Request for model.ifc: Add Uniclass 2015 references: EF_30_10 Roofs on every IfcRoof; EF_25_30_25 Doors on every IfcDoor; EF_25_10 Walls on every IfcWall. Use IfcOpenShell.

First a look at what the model holds.

```python
import ifcopenshell

model = ifcopenshell.open("model.ifc")
print(model.schema)
print("classifications:", [c.Name for c in model.by_type("IfcClassification")])
for ifc_class in ("IfcDoor", "IfcRoof", "IfcStair", "IfcWall", "IfcWindow"):
    print(ifc_class, len(model.by_type(ifc_class)))
```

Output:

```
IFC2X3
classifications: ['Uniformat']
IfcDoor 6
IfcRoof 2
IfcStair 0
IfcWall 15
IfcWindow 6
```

```python
import ifcopenshell
import ifcopenshell.api.classification

model = ifcopenshell.open("model.ifc")

# IFC2X3 requires Source and Edition and has no link from the project to the system.
system = model.create_entity("IfcClassification", Source="NBS", Edition="2015", Name="Uniclass 2015")

codes = {
    "IfcRoof": ("EF_30_10", "Roofs"),
    "IfcDoor": ("EF_25_30_25", "Doors"),
    "IfcWall": ("EF_25_10", "Walls"),
}
for ifc_class, (code, name) in codes.items():
    products = model.by_type(ifc_class)
    ifcopenshell.api.classification.add_reference(
        model, products=products, classification=system, identification=code, name=name
    )
    print(code, len(products))

model.write("model_v2.ifc")
```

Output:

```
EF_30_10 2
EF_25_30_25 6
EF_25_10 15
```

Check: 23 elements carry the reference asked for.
